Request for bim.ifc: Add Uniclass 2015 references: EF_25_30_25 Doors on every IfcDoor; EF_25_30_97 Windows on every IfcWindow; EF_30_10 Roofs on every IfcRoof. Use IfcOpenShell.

First a look at what the model holds.

```python
import ifcopenshell

model = ifcopenshell.open("bim.ifc")
print(model.schema)
print("classifications:", [c.Name for c in model.by_type("IfcClassification")])
for ifc_class in ("IfcDoor", "IfcRoof", "IfcStair", "IfcWall", "IfcWindow"):
    print(ifc_class, len(model.by_type(ifc_class)))
```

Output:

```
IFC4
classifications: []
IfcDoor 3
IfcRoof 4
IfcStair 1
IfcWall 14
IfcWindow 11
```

```python
import ifcopenshell
import ifcopenshell.api.classification

model = ifcopenshell.open("bim.ifc")

system = ifcopenshell.api.classification.add_classification(model, classification="Uniclass 2015")

codes = {
    "IfcDoor": ("EF_25_30_25", "Doors"),
    "IfcWindow": ("EF_25_30_97", "Windows"),
    "IfcRoof": ("EF_30_10", "Roofs"),
}
for ifc_class, (code, name) in codes.items():
    products = model.by_type(ifc_class)
    ifcopenshell.api.classification.add_reference(
        model, products=products, classification=system, identification=code, name=name
    )
    print(code, len(products))

model.write("bim-out.ifc")
```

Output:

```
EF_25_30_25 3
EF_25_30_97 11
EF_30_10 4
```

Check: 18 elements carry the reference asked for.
